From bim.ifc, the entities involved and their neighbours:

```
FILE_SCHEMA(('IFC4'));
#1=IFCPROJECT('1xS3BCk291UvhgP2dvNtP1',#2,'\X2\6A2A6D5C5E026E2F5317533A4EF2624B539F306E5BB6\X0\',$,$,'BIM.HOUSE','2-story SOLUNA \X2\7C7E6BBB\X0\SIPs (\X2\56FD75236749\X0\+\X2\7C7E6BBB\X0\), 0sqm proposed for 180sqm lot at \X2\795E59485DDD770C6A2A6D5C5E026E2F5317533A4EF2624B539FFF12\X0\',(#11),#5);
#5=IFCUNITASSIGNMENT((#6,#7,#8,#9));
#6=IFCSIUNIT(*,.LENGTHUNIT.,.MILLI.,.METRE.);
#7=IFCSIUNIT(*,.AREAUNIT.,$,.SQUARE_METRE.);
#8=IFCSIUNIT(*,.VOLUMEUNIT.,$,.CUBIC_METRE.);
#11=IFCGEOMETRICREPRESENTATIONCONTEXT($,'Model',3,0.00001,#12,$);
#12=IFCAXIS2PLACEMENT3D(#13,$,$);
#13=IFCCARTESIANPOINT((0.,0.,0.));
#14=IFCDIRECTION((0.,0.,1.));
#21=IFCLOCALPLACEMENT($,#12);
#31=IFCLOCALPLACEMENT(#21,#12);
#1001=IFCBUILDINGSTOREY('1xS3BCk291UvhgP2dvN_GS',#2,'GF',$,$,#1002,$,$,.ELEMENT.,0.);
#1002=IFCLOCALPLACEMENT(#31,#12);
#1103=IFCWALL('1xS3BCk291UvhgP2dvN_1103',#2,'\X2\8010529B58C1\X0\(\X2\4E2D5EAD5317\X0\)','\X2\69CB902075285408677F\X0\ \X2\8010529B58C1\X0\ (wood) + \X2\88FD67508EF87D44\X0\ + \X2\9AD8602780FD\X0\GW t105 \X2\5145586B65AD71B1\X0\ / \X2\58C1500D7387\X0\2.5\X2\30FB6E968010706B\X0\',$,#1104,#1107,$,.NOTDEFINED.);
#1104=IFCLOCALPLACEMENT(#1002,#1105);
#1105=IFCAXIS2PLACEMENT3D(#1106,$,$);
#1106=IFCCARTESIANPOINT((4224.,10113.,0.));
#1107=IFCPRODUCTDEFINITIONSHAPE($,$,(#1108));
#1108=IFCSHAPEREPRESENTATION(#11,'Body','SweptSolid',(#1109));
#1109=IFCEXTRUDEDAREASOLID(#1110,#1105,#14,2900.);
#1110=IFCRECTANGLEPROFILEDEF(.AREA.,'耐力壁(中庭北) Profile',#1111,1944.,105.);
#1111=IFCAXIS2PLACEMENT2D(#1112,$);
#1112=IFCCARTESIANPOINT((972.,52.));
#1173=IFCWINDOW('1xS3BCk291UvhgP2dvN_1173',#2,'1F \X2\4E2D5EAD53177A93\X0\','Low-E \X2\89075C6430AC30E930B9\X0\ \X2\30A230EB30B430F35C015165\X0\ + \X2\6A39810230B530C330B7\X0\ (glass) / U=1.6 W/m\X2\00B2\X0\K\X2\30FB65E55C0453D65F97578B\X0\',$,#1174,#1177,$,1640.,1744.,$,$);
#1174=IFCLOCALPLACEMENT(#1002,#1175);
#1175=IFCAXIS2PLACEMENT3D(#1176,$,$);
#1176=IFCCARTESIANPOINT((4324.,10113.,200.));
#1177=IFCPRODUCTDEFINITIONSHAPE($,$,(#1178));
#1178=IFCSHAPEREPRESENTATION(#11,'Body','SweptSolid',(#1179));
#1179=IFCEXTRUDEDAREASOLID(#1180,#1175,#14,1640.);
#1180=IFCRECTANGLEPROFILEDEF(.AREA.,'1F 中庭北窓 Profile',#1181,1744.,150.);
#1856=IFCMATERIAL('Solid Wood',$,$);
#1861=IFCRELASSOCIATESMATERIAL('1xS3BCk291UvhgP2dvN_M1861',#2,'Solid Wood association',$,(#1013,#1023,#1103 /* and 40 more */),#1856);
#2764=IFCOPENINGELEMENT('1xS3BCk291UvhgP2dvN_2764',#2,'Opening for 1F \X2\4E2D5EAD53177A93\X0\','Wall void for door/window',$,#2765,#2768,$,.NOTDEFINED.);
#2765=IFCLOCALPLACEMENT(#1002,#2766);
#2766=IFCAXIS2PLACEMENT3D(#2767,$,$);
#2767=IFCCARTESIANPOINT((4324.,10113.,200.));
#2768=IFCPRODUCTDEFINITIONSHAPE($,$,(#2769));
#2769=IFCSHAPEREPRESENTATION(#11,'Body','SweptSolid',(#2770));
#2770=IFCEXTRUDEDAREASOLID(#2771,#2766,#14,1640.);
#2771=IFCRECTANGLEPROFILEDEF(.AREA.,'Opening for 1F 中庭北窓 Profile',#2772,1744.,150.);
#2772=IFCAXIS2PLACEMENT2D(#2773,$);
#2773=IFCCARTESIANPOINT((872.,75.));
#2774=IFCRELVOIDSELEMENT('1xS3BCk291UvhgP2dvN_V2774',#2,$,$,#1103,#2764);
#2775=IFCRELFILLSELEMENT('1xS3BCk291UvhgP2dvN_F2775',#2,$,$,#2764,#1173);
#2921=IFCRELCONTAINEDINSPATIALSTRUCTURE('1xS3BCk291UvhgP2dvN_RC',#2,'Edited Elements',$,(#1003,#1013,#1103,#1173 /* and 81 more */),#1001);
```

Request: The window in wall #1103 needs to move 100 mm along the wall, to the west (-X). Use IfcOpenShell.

```python
import ifcopenshell
import ifcopenshell.api.geometry
import ifcopenshell.util.placement

model = ifcopenshell.open("bim.ifc")

window = model.by_id(1173)
opening = window.FillsVoids[0].RelatingOpeningElement
wall = opening.VoidsElements[0].RelatingBuildingElement

wall_matrix = ifcopenshell.util.placement.get_local_placement(wall.ObjectPlacement)
shift = wall_matrix[:3, 0] * -100.0
before = ifcopenshell.util.placement.get_local_placement(window.ObjectPlacement)[:3, 3].copy()

# The window is not placed relative to its opening, so move both.
for product in (opening, window):
    matrix = ifcopenshell.util.placement.get_local_placement(product.ObjectPlacement)
    matrix[:3, 3] += shift
    ifcopenshell.api.geometry.edit_object_placement(model, product=product, matrix=matrix, is_si=False)

after = ifcopenshell.util.placement.get_local_placement(window.ObjectPlacement)[:3, 3]
print("window moved by", (after - before).round(3) + 0.0)

model.write("bim_rev.ifc")
```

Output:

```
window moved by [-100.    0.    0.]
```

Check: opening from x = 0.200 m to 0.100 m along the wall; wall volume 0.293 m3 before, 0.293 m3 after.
